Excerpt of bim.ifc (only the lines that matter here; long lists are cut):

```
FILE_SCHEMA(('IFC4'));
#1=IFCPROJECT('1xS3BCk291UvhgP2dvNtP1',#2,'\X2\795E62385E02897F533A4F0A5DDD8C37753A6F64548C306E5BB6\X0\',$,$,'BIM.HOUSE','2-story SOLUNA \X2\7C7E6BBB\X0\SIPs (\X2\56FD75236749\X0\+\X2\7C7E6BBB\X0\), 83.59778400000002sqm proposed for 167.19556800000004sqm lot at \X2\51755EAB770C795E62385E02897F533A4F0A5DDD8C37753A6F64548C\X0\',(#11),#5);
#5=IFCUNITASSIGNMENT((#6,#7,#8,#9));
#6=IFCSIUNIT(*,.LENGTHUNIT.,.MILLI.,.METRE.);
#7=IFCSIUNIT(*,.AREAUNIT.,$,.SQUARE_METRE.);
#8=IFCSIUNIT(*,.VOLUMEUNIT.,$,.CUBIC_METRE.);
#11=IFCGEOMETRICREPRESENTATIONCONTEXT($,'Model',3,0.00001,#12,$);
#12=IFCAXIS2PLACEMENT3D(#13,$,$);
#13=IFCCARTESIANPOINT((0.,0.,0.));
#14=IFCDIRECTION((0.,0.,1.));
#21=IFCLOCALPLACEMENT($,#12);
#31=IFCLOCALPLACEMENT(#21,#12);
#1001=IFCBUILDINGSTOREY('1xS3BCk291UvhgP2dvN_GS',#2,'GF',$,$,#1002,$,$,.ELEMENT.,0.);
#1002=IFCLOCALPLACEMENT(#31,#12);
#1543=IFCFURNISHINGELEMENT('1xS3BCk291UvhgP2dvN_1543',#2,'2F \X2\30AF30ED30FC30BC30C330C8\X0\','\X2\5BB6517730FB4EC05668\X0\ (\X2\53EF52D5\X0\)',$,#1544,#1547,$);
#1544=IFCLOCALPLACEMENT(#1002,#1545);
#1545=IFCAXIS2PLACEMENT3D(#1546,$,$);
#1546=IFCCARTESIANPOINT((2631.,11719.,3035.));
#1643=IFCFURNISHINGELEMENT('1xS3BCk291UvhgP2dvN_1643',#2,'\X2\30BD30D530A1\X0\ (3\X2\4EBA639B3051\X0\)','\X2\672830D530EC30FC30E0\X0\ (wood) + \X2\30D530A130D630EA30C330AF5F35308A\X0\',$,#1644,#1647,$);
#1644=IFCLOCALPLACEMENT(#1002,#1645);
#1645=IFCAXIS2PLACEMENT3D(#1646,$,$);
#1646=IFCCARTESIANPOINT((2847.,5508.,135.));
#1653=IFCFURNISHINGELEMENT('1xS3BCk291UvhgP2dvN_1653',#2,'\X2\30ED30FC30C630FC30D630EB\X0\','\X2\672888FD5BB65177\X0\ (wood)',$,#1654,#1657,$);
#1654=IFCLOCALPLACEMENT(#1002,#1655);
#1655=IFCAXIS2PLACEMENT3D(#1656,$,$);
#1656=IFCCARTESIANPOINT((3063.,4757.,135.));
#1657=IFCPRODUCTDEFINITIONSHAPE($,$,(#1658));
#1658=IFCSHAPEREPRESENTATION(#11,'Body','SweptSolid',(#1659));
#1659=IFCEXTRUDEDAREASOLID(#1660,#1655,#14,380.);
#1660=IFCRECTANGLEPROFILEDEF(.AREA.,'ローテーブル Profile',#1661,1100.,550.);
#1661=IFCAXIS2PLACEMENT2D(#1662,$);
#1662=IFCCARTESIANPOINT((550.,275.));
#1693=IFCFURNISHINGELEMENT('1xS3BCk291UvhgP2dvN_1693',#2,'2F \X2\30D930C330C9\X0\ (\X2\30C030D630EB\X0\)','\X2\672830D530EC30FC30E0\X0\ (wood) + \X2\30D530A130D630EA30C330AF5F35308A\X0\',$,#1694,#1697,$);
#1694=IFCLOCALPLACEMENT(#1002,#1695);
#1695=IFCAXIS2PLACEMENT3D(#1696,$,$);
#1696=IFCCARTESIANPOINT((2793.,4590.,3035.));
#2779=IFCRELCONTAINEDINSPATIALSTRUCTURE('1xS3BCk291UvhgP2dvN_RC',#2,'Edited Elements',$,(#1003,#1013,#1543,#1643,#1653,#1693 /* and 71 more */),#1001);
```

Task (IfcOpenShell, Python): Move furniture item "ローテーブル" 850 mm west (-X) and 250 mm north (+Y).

```python
import ifcopenshell
import ifcopenshell.api.geometry
import ifcopenshell.util.placement

model = ifcopenshell.open("bim.ifc")

item = model.by_guid("1xS3BCk291UvhgP2dvN_1653")
matrix = ifcopenshell.util.placement.get_local_placement(item.ObjectPlacement)
matrix[0, 3] -= 850.0
matrix[1, 3] += 250.0
ifcopenshell.api.geometry.edit_object_placement(model, product=item, matrix=matrix, is_si=False)

print(ifcopenshell.util.placement.get_local_placement(item.ObjectPlacement).round(3) + 0.0)

model.write("bim_rev.ifc")
```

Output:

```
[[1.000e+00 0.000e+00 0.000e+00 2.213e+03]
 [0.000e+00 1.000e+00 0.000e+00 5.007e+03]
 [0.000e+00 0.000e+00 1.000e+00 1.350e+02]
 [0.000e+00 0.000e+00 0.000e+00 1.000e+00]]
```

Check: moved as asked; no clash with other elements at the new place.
